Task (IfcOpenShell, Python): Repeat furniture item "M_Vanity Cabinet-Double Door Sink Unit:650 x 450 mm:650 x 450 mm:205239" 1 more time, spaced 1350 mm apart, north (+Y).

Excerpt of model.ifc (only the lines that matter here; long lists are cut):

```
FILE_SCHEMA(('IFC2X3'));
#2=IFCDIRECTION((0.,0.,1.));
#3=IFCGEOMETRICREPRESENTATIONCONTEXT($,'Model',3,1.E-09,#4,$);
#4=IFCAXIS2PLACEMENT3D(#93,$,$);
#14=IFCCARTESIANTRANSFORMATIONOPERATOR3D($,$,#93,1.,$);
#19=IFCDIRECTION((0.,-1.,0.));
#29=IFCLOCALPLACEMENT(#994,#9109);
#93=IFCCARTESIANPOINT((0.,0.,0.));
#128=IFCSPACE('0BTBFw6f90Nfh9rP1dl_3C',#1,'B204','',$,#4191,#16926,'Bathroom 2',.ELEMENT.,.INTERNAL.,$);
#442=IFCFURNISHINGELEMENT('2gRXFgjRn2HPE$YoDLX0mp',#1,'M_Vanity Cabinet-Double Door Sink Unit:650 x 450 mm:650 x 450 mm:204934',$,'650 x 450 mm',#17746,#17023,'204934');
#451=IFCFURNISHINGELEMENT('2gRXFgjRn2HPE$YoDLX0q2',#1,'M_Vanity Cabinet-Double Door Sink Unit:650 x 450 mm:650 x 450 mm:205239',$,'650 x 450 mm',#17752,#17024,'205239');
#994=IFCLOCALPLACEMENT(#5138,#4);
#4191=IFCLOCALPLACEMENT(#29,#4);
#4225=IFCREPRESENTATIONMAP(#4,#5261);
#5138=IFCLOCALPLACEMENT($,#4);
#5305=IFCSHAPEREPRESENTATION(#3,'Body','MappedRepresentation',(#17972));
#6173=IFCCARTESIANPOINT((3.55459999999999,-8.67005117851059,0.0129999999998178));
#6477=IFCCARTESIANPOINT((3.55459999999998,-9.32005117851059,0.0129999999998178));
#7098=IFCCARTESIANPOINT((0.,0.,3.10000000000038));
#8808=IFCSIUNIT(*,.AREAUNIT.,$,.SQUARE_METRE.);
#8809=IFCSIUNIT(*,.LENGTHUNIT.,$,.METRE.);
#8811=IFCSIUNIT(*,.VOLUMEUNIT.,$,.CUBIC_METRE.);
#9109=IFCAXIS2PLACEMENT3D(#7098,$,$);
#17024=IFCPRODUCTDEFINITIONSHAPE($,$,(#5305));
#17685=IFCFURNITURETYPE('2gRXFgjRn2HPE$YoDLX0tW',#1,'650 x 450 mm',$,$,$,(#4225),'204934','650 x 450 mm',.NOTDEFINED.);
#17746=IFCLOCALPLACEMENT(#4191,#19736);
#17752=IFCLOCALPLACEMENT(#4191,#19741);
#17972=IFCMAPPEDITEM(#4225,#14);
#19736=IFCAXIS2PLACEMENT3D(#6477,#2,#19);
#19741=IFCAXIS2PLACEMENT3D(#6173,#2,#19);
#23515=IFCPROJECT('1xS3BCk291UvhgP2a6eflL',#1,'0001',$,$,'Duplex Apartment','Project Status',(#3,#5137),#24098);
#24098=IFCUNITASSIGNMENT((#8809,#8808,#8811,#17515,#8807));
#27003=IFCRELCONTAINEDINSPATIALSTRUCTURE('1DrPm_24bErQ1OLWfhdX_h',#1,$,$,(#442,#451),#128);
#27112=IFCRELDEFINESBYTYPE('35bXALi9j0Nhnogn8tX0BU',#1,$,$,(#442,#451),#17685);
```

```python
import numpy as np
import ifcopenshell
import ifcopenshell.api.geometry
import ifcopenshell.api.root
import ifcopenshell.util.element
import ifcopenshell.util.placement

model = ifcopenshell.open("model.ifc")


def reuse_history(source, copy):
    """copy_class also copies each property set's owner history, people and application; keep the originals."""
    for rel in copy.IsDefinedBy:
        if rel.is_a("IfcRelDefinesByProperties") and (history := rel.RelatingPropertyDefinition.OwnerHistory):
            rel.RelatingPropertyDefinition.OwnerHistory = source.OwnerHistory
            ifcopenshell.util.element.remove_deep2(model, history)


source = model.by_id(451)
base = ifcopenshell.util.placement.get_local_placement(source.ObjectPlacement)
step = np.array([0.0, 1.0, 0.0]) * 1.35

for i in range(1, 2):
    copy = ifcopenshell.api.root.copy_class(model, product=source)
    copy.Representation = ifcopenshell.util.element.copy_deep(
        model, source.Representation, exclude=["IfcGeometricRepresentationContext", "IfcRepresentationMap"]
    )
    copy.Name = "M_Vanity Cabinet-Double Door Sink Unit:650 x 450 mm:650 x 450 mm"
    copy.Tag = None
    reuse_history(source, copy)
    matrix = base.copy()
    matrix[:3, 3] += i * step
    print("added at", matrix[:3, 3].round(3) + 0.0)
    ifcopenshell.api.geometry.edit_object_placement(model, product=copy, matrix=matrix, is_si=False)

model.write("model_rev.ifc")
```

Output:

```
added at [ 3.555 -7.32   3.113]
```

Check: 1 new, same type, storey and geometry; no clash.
